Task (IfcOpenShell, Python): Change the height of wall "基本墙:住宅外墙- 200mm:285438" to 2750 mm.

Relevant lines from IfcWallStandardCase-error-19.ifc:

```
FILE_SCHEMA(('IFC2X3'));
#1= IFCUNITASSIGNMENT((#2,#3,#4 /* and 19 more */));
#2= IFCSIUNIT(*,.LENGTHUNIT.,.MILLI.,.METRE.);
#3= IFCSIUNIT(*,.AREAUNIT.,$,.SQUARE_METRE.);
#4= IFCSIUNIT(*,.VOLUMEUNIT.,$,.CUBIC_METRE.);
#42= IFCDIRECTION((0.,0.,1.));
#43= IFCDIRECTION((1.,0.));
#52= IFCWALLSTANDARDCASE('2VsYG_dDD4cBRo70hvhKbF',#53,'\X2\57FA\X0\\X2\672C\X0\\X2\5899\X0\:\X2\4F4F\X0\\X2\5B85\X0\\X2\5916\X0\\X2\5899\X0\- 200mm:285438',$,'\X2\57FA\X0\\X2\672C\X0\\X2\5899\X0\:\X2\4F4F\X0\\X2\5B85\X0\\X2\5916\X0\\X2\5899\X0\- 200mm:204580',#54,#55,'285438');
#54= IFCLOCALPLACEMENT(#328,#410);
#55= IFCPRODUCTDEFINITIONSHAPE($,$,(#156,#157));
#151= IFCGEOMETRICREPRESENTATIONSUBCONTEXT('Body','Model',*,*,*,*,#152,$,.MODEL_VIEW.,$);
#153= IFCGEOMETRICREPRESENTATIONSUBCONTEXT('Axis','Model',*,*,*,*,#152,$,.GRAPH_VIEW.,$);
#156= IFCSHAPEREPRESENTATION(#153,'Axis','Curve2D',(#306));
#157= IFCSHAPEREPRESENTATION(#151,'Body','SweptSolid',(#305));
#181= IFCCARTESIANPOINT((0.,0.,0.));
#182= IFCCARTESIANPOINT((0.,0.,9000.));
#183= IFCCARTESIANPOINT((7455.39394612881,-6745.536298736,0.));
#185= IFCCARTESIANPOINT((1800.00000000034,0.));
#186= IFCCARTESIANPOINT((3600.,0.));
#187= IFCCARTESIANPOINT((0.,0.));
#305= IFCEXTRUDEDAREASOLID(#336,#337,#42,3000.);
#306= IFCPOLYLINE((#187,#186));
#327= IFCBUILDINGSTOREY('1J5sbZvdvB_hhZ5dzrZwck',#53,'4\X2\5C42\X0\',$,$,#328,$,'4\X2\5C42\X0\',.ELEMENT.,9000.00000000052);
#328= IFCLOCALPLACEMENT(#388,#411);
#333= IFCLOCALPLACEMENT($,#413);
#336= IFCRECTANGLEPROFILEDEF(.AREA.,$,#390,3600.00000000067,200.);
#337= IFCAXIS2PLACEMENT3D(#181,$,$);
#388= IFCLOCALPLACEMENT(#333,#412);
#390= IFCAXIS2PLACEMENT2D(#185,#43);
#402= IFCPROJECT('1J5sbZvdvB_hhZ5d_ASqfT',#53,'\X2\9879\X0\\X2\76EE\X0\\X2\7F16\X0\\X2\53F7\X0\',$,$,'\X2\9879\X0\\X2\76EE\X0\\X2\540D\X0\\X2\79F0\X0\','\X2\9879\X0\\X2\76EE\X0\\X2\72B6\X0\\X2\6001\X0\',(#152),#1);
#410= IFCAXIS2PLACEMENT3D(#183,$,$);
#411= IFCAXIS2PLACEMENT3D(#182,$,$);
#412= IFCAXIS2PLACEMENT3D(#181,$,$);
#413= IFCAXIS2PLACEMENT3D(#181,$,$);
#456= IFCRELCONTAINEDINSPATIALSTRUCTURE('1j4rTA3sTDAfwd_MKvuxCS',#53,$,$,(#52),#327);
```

```python
import ifcopenshell
import ifcopenshell.geom
import ifcopenshell.util.representation
import ifcopenshell.util.shape
import ifcopenshell.util.unit

model = ifcopenshell.open("IfcWallStandardCase-error-19.ifc")
unit_scale = ifcopenshell.util.unit.calculate_unit_scale(model)
settings = ifcopenshell.geom.settings()


def volume(element):
    """Net volume in cubic metres, openings subtracted."""
    shape = ifcopenshell.geom.create_shape(settings, element)
    return ifcopenshell.util.shape.get_volume(shape.geometry)


wall = model.by_guid("2VsYG_dDD4cBRo70hvhKbF")
before = volume(wall)

body = ifcopenshell.util.representation.get_representation(wall, "Model", "Body")
solid = body.Items[0]
old_height = solid.Depth
solid.Depth = 2.75 / unit_scale
after = volume(wall)

print(f"height {old_height:g} -> {solid.Depth:g}, volume {before:.3f} -> {after:.3f} m3")

model.write("IfcWallStandardCase-error-19_edited.ifc")
```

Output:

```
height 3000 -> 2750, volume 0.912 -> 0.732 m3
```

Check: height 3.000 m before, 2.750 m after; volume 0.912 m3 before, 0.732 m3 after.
